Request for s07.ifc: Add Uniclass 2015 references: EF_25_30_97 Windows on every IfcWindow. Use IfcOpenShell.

First a look at what the model holds.

```python
import ifcopenshell

model = ifcopenshell.open("s07.ifc")
print(model.schema)
print("classifications:", [c.Name for c in model.by_type("IfcClassification")])
for ifc_class in ("IfcDoor", "IfcRoof", "IfcStair", "IfcWall", "IfcWindow"):
    print(ifc_class, len(model.by_type(ifc_class)))
```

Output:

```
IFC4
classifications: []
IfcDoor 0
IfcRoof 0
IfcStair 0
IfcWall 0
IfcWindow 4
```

```python
import ifcopenshell
import ifcopenshell.api.classification

model = ifcopenshell.open("s07.ifc")

system = ifcopenshell.api.classification.add_classification(model, classification="Uniclass 2015")

codes = {
    "IfcWindow": ("EF_25_30_97", "Windows"),
}
for ifc_class, (code, name) in codes.items():
    products = model.by_type(ifc_class)
    ifcopenshell.api.classification.add_reference(
        model, products=products, classification=system, identification=code, name=name
    )
    print(code, len(products))

model.write("s07_edited.ifc")
```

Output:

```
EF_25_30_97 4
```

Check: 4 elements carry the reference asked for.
